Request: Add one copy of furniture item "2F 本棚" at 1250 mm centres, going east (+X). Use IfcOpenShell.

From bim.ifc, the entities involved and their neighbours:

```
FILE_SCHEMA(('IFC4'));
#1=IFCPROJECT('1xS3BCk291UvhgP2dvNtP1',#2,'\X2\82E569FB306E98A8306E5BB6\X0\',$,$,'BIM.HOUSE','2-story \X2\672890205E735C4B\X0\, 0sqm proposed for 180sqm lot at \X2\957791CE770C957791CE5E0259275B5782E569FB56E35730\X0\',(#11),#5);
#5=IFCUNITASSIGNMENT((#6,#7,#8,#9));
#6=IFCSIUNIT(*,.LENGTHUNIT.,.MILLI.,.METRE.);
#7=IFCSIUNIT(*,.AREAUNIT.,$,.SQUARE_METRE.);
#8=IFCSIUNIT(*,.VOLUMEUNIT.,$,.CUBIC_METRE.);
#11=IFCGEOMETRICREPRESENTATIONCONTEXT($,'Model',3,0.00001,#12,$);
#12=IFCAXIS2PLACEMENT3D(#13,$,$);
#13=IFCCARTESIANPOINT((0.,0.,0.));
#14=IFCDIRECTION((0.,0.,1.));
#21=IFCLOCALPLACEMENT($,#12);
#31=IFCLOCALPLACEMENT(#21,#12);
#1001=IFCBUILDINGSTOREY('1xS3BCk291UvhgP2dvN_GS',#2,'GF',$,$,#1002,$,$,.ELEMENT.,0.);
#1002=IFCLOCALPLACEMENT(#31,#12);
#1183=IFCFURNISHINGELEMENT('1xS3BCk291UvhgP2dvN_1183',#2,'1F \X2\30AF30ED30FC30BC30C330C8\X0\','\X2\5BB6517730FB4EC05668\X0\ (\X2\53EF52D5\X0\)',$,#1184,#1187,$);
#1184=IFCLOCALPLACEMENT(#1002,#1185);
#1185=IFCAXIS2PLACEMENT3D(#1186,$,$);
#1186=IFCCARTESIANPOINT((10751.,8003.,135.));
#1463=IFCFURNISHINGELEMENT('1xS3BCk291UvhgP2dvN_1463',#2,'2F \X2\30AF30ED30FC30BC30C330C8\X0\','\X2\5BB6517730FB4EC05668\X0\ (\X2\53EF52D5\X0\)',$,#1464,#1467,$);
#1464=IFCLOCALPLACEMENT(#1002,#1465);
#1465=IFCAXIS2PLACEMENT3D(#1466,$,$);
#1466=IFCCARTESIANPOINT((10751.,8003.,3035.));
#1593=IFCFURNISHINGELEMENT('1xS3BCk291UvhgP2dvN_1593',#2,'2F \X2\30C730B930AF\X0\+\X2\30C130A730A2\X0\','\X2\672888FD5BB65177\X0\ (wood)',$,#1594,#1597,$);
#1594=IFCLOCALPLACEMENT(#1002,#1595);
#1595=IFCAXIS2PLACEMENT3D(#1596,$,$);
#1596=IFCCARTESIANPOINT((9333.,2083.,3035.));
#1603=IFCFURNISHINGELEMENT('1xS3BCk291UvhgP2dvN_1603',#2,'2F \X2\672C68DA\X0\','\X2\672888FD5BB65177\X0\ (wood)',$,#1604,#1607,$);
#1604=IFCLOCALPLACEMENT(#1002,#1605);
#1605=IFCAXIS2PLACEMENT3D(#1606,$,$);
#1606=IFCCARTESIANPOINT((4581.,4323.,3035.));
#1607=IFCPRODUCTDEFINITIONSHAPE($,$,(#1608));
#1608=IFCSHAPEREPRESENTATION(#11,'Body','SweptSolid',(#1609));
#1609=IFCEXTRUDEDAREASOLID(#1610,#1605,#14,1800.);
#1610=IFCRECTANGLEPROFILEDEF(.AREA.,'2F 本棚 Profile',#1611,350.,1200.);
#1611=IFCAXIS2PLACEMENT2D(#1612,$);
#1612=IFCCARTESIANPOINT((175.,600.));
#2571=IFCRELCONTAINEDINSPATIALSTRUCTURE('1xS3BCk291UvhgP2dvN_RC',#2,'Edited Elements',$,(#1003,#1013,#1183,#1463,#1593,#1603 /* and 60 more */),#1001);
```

```python
import numpy as np
import ifcopenshell
import ifcopenshell.api.geometry
import ifcopenshell.api.root
import ifcopenshell.util.element
import ifcopenshell.util.placement
import ifcopenshell.util.unit

model = ifcopenshell.open("bim.ifc")
unit_scale = ifcopenshell.util.unit.calculate_unit_scale(model)


def reuse_history(source, copy):
    """copy_class also copies each property set's owner history, people and application; keep the originals."""
    for rel in copy.IsDefinedBy:
        if rel.is_a("IfcRelDefinesByProperties") and (history := rel.RelatingPropertyDefinition.OwnerHistory):
            rel.RelatingPropertyDefinition.OwnerHistory = source.OwnerHistory
            ifcopenshell.util.element.remove_deep2(model, history)


source = model.by_guid("1xS3BCk291UvhgP2dvN_1603")
base = ifcopenshell.util.placement.get_local_placement(source.ObjectPlacement)
step = np.array([1.0, 0.0, 0.0]) * 1.25 / unit_scale

for i in range(1, 2):
    copy = ifcopenshell.api.root.copy_class(model, product=source)
    copy.Representation = ifcopenshell.util.element.copy_deep(
        model, source.Representation, exclude=["IfcGeometricRepresentationContext", "IfcRepresentationMap"]
    )
    reuse_history(source, copy)
    matrix = base.copy()
    matrix[:3, 3] += i * step
    print("added at", matrix[:3, 3].round(3) + 0.0)
    ifcopenshell.api.geometry.edit_object_placement(model, product=copy, matrix=matrix, is_si=False)

model.write("bim_updated.ifc")
```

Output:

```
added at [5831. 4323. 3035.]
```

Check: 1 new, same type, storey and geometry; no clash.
